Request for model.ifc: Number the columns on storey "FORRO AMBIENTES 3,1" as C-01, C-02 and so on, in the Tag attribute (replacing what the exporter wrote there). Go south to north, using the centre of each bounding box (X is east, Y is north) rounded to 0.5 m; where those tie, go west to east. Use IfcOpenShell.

First a look at what the model holds.

```python
import ifcopenshell
import ifcopenshell.util.element
import ifcopenshell.util.placement

model = ifcopenshell.open("model.ifc")
print(model.schema)
storey = next(s for s in model.by_type("IfcBuildingStorey") if s.Name == "FORRO AMBIENTES 3,1")
columns = [e for e in ifcopenshell.util.element.get_decomposition(storey) if e.is_a("IfcColumn")]
for e in sorted(columns, key=lambda e: e.id()):
    origin = ifcopenshell.util.placement.get_local_placement(e.ObjectPlacement)[:3, 3]
    print(e.id(), e.Tag, e.Name, origin.round(2) + 0.0, sep=" | ")
```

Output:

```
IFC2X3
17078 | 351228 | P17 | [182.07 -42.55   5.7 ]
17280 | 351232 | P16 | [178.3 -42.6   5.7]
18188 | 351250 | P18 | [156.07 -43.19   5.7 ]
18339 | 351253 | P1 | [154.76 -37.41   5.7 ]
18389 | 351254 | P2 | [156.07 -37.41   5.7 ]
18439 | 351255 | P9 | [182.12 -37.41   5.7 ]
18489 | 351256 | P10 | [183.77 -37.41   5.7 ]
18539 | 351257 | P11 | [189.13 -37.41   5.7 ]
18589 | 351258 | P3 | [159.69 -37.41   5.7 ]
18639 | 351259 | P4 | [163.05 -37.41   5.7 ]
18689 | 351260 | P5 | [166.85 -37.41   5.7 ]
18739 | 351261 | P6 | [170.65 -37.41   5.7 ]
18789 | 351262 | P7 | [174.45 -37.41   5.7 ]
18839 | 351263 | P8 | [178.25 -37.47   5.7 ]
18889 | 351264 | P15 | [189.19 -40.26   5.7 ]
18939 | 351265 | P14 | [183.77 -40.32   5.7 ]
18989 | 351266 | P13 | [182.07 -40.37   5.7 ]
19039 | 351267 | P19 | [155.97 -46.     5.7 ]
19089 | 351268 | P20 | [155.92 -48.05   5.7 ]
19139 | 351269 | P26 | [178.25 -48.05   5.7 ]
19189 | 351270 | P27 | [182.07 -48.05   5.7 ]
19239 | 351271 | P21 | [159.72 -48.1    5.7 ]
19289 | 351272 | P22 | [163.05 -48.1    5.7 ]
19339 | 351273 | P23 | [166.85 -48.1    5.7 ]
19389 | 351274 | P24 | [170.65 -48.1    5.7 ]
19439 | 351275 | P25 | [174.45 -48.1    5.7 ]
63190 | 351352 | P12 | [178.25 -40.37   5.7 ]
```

```python
import ifcopenshell
import ifcopenshell.geom
import ifcopenshell.util.element
import ifcopenshell.util.shape

model = ifcopenshell.open("model.ifc")
settings = ifcopenshell.geom.settings()
settings.set("use-world-coords", True)


def centre(element):
    shape = ifcopenshell.geom.create_shape(settings, element)
    return ifcopenshell.util.shape.get_bbox_centroid(shape.geometry)


storey = next(s for s in model.by_type("IfcBuildingStorey") if s.Name == "FORRO AMBIENTES 3,1")
columns = [e for e in ifcopenshell.util.element.get_decomposition(storey) if e.is_a("IfcColumn")]

# Insertion points can sit at a corner or the storey origin, so sort by the geometry (in metres).
centres = {e: centre(e) for e in columns}
columns.sort(key=lambda e: (round(centres[e][1] / 0.5), centres[e][0]))

for i, e in enumerate(columns, start=1):
    number = f"C-{i:02d}"
    e.Tag = number
    print(e.id(), number)

model.write("model_edited.ifc")
```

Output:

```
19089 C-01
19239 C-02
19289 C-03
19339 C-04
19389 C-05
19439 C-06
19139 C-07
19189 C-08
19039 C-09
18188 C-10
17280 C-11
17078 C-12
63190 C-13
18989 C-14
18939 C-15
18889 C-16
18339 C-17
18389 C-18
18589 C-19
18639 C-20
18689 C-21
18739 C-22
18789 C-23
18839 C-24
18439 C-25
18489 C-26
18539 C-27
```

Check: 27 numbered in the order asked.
